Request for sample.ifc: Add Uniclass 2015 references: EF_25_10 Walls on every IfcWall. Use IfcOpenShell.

First a look at what the model holds.

```python
import ifcopenshell

model = ifcopenshell.open("sample.ifc")
print(model.schema)
print("classifications:", [c.Name for c in model.by_type("IfcClassification")])
for ifc_class in ("IfcDoor", "IfcRoof", "IfcStair", "IfcWall", "IfcWindow"):
    print(ifc_class, len(model.by_type(ifc_class)))
```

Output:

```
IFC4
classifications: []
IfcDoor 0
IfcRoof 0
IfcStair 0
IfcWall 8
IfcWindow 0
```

```python
import ifcopenshell
import ifcopenshell.api.classification

model = ifcopenshell.open("sample.ifc")

system = ifcopenshell.api.classification.add_classification(model, classification="Uniclass 2015")

codes = {
    "IfcWall": ("EF_25_10", "Walls"),
}
for ifc_class, (code, name) in codes.items():
    products = model.by_type(ifc_class)
    ifcopenshell.api.classification.add_reference(
        model, products=products, classification=system, identification=code, name=name
    )
    print(code, len(products))

model.write("sample_rev.ifc")
```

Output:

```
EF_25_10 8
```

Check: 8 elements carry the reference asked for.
